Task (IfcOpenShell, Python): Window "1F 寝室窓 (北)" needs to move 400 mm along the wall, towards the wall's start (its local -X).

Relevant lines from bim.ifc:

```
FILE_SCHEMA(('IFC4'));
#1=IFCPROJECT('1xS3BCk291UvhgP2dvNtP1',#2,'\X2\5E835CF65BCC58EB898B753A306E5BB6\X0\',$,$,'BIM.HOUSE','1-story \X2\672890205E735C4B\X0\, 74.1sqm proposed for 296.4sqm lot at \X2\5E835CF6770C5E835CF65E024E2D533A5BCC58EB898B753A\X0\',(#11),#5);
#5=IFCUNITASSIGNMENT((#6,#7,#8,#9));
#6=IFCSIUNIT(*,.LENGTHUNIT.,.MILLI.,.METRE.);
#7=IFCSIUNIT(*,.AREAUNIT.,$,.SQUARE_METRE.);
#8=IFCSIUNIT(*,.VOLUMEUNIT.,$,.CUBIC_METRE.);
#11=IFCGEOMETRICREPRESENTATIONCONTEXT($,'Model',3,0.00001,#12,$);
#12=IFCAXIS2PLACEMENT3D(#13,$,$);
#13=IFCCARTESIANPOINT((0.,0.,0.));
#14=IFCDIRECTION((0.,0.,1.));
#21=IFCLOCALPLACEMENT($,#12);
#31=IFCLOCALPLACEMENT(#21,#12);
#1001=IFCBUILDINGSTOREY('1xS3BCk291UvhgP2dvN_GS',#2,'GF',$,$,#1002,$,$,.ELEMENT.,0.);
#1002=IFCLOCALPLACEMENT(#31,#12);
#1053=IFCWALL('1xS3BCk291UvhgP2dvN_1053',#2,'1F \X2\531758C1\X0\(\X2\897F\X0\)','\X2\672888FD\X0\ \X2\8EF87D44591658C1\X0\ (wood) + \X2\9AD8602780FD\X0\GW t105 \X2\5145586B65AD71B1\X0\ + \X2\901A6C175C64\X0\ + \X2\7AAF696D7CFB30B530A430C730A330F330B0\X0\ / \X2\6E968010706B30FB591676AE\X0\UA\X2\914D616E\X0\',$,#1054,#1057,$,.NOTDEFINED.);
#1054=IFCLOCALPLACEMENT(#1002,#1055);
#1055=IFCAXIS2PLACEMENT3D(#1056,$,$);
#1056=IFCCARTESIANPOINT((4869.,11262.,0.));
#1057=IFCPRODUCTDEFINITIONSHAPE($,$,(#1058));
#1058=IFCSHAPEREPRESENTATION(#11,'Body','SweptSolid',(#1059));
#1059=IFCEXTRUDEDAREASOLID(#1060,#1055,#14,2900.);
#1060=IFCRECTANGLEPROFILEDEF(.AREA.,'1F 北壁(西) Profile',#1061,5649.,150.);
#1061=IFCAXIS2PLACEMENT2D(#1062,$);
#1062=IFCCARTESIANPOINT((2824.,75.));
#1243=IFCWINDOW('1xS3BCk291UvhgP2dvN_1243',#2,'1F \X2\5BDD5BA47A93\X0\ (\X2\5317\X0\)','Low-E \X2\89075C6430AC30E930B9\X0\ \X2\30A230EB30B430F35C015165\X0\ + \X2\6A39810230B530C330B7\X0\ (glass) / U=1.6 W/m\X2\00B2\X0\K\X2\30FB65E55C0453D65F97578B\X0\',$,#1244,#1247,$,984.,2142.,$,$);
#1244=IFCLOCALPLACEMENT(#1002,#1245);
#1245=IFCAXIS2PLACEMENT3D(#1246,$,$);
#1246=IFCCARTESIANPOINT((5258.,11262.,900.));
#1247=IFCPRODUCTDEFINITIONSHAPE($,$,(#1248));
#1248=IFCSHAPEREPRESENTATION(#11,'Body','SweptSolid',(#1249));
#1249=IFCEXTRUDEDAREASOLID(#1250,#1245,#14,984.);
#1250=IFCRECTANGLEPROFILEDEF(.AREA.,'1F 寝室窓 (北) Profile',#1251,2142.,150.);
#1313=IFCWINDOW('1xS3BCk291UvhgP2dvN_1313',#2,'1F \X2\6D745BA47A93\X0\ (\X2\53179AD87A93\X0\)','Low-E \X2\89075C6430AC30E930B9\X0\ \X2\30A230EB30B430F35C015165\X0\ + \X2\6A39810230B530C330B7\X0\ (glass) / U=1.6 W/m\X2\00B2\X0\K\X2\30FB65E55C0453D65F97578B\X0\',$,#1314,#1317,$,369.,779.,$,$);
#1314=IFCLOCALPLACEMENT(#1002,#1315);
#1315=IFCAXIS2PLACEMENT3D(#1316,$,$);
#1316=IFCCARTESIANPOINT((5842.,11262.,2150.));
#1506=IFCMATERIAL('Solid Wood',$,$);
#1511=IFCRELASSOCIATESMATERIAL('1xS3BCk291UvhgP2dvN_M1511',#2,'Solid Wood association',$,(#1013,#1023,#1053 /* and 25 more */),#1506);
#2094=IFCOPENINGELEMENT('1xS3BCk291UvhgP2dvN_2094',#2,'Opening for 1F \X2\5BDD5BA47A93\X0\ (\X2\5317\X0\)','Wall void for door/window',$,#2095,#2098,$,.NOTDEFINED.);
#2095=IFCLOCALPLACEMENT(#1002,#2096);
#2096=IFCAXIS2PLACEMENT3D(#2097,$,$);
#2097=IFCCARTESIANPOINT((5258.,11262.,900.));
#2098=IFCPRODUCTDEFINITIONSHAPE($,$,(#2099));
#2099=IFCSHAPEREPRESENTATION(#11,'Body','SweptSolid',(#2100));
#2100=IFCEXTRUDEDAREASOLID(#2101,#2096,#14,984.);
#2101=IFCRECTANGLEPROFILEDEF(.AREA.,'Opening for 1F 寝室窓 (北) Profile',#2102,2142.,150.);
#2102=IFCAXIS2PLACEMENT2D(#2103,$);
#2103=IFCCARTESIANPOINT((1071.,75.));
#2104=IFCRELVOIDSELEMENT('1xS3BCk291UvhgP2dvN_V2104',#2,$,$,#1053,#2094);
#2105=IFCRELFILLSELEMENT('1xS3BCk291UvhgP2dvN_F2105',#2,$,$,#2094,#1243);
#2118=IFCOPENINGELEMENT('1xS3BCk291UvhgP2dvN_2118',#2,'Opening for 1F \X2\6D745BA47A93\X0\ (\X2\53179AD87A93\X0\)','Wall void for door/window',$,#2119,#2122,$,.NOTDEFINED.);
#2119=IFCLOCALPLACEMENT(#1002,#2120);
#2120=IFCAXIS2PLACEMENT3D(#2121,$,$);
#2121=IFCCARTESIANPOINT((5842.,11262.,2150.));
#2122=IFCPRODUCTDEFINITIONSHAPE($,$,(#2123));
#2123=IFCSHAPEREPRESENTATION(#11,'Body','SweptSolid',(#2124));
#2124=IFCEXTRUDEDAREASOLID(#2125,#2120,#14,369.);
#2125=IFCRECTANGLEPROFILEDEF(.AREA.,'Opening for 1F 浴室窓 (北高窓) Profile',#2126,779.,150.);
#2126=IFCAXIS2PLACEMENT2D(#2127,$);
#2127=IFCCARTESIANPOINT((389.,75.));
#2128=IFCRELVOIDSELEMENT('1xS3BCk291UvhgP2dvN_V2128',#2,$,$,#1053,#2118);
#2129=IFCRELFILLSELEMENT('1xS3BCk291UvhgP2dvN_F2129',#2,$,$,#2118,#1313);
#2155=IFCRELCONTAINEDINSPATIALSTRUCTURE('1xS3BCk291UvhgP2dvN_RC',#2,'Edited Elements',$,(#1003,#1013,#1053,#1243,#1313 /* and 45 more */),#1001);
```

```python
import ifcopenshell
import ifcopenshell.api.geometry
import ifcopenshell.util.placement

model = ifcopenshell.open("bim.ifc")

window = model.by_guid("1xS3BCk291UvhgP2dvN_1243")
opening = window.FillsVoids[0].RelatingOpeningElement
wall = opening.VoidsElements[0].RelatingBuildingElement

wall_matrix = ifcopenshell.util.placement.get_local_placement(wall.ObjectPlacement)
shift = wall_matrix[:3, 0] * -400.0
before = ifcopenshell.util.placement.get_local_placement(window.ObjectPlacement)[:3, 3].copy()

# The window is not placed relative to its opening, so move both.
for product in (opening, window):
    matrix = ifcopenshell.util.placement.get_local_placement(product.ObjectPlacement)
    matrix[:3, 3] += shift
    ifcopenshell.api.geometry.edit_object_placement(model, product=product, matrix=matrix, is_si=False)

after = ifcopenshell.util.placement.get_local_placement(window.ObjectPlacement)[:3, 3]
print("window moved by", (after - before).round(3) + 0.0)

model.write("bim-out.ifc")
```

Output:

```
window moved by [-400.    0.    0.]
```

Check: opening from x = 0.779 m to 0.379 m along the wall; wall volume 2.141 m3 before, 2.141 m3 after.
